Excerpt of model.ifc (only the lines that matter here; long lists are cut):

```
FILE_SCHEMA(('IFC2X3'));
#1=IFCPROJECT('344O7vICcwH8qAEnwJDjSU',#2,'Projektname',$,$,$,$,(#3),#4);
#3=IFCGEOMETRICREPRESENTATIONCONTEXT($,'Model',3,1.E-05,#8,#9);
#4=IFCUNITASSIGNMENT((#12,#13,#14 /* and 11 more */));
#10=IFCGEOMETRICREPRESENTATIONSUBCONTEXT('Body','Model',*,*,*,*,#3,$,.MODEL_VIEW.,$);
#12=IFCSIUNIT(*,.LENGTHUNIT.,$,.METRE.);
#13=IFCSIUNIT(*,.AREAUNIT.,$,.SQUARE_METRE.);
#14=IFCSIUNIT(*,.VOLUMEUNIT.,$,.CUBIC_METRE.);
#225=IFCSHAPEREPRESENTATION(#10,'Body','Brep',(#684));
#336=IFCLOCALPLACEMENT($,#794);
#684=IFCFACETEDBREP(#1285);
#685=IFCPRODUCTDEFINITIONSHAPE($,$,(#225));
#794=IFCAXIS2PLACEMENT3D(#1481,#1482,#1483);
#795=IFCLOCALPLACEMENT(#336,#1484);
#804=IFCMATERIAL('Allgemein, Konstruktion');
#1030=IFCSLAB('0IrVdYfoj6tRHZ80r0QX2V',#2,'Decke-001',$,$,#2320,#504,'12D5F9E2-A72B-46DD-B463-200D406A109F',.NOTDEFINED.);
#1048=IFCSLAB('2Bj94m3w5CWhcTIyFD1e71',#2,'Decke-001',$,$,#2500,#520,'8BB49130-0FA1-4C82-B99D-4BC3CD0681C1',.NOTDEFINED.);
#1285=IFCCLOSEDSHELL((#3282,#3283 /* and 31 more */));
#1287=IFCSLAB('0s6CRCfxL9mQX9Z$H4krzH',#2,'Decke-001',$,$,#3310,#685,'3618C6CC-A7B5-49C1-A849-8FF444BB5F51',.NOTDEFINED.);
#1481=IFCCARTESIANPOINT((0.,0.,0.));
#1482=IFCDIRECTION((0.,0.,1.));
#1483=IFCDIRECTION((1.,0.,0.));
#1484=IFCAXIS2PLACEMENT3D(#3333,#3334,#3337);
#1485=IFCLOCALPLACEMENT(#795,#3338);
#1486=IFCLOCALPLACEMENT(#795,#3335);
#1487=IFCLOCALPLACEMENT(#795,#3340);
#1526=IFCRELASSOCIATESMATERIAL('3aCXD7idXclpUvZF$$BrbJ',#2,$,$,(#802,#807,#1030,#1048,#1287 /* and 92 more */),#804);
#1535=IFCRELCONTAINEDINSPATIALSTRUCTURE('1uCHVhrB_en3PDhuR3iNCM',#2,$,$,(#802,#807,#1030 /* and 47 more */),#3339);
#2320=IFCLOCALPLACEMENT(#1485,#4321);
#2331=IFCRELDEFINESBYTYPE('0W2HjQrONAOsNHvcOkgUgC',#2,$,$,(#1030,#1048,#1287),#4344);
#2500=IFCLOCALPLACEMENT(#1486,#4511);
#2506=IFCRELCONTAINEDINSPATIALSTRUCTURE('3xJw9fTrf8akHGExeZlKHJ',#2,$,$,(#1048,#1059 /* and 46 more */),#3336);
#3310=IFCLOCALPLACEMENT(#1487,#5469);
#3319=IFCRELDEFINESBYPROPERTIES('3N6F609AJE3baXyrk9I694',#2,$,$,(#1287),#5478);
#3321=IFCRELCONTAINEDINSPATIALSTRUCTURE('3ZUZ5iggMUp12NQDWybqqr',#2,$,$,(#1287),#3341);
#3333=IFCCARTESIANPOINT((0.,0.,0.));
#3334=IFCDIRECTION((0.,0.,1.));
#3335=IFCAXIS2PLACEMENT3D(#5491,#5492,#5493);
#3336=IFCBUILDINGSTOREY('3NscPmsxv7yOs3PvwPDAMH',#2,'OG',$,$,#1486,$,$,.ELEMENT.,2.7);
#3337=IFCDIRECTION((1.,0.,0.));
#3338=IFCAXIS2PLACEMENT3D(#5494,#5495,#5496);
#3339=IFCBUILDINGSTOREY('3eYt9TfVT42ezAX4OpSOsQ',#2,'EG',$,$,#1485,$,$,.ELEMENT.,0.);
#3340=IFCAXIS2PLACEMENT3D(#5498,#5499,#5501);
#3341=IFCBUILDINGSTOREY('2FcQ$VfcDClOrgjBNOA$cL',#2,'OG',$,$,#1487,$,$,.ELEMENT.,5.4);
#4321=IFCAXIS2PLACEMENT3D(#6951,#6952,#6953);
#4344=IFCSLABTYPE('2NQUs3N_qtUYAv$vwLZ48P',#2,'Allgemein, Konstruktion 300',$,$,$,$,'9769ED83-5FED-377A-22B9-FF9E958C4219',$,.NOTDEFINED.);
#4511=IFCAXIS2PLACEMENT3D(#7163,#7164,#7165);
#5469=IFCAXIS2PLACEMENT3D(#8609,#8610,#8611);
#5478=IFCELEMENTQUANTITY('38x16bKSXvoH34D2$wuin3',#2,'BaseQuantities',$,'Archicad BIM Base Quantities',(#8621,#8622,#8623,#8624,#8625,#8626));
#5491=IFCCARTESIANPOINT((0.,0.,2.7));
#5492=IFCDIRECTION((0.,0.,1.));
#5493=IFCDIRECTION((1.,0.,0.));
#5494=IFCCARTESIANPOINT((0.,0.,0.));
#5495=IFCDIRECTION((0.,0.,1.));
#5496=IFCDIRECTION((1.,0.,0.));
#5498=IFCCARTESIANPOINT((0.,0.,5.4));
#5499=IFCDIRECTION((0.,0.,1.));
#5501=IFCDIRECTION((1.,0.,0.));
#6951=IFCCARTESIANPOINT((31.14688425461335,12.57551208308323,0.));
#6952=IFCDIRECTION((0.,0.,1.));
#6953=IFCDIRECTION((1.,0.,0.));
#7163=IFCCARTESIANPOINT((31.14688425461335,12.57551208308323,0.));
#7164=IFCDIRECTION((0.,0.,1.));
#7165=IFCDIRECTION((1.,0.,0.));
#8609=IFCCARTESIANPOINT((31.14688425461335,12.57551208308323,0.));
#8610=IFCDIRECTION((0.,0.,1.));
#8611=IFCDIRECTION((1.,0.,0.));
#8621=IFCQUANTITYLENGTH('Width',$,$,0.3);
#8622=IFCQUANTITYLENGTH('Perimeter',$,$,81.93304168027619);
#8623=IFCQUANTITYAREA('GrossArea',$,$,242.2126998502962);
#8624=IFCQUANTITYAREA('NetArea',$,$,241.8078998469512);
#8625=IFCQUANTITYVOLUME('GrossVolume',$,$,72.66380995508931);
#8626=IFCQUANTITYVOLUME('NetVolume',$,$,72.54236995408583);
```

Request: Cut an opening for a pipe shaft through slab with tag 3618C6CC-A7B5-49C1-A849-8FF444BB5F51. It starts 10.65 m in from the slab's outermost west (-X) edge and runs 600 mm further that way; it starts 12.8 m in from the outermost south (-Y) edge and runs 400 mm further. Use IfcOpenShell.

```python
import numpy as np
import ifcopenshell
import ifcopenshell.api.feature
import ifcopenshell.api.geometry
import ifcopenshell.api.pset
import ifcopenshell.api.root
import ifcopenshell.geom
import ifcopenshell.util.element
import ifcopenshell.util.placement
import ifcopenshell.util.representation
import ifcopenshell.util.shape
import ifcopenshell.util.unit

model = ifcopenshell.open("model.ifc")
unit_scale = ifcopenshell.util.unit.calculate_unit_scale(model)
area_scale = ifcopenshell.util.unit.calculate_unit_scale(model, "AREAUNIT")
volume_scale = ifcopenshell.util.unit.calculate_unit_scale(model, "VOLUMEUNIT")
settings = ifcopenshell.geom.settings()


def volume(element):
    """Net volume in cubic metres, openings subtracted."""
    shape = ifcopenshell.geom.create_shape(settings, element)
    return ifcopenshell.util.shape.get_volume(shape.geometry)


slab = model.by_guid("0s6CRCfxL9mQX9Z$H4krzH")
before = volume(slab)

# Extent in the slab's own axes, in metres. The edges named are its -X and -Y sides.
slab_shape = ifcopenshell.geom.create_shape(settings, slab)
vertices = ifcopenshell.util.shape.get_vertices(slab_shape.geometry)
x_min, y_min, bottom = vertices.min(axis=0)
top = vertices[:, 2].max()

opening = ifcopenshell.api.root.create_entity(model, ifc_class="IfcOpeningElement", name="Pipe shaft opening")
context = ifcopenshell.util.representation.get_context(model, "Model", "Body", "MODEL_VIEW")
width, depth = 0.6, 0.4
outline = [(0.0, 0.0), (width, 0.0), (width, depth), (0.0, depth), (0.0, 0.0)]
# Overshoot both faces by 50 mm so the cut is clean.
shape = ifcopenshell.api.geometry.add_slab_representation(
    model, context=context, depth=top - bottom + 0.1, polyline=outline
)
ifcopenshell.api.geometry.assign_representation(model, product=opening, representation=shape)

matrix = ifcopenshell.util.placement.get_local_placement(slab.ObjectPlacement)
matrix[:, 3] = matrix @ np.append(np.array([x_min + 10.65, y_min + 12.8, bottom - 0.05]) / unit_scale, 1.0)
ifcopenshell.api.geometry.edit_object_placement(model, product=opening, matrix=matrix, is_si=False)
ifcopenshell.api.feature.add_feature(model, feature=opening, element=slab)

after = volume(slab)

# Update the slab's stored quantities.
qto = model.by_id(ifcopenshell.util.element.get_pset(slab, "BaseQuantities", should_inherit=False)["id"])
ifcopenshell.api.pset.edit_qto(model, qto=qto, properties={
    "NetArea": after / (top - bottom) / area_scale,
    "NetVolume": after / volume_scale,
})

print(f"slab volume {before:.3f} -> {after:.3f} m3")

model.write("model_v2.ifc")
```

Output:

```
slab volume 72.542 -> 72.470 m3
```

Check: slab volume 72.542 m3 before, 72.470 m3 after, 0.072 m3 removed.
